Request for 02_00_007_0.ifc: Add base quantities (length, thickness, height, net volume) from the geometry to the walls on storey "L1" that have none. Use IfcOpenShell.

First a look at what the model holds.

```python
import ifcopenshell
import ifcopenshell.util.element
import ifcopenshell.util.unit

model = ifcopenshell.open("02_00_007_0.ifc")
print(model.schema)
for unit_type in ("LENGTHUNIT", "AREAUNIT", "VOLUMEUNIT"):
    print(unit_type, ifcopenshell.util.unit.calculate_unit_scale(model, unit_type))
storey = next(s for s in model.by_type("IfcBuildingStorey") if s.Name == "L1")
walls = [e for e in ifcopenshell.util.element.get_decomposition(storey) if e.is_a("IfcWall")]
for e in sorted(walls, key=lambda e: e.id()):
    print(e.id(), e.is_a(), e.Name, list(ifcopenshell.util.element.get_psets(e, qtos_only=True)), sep=" | ")
```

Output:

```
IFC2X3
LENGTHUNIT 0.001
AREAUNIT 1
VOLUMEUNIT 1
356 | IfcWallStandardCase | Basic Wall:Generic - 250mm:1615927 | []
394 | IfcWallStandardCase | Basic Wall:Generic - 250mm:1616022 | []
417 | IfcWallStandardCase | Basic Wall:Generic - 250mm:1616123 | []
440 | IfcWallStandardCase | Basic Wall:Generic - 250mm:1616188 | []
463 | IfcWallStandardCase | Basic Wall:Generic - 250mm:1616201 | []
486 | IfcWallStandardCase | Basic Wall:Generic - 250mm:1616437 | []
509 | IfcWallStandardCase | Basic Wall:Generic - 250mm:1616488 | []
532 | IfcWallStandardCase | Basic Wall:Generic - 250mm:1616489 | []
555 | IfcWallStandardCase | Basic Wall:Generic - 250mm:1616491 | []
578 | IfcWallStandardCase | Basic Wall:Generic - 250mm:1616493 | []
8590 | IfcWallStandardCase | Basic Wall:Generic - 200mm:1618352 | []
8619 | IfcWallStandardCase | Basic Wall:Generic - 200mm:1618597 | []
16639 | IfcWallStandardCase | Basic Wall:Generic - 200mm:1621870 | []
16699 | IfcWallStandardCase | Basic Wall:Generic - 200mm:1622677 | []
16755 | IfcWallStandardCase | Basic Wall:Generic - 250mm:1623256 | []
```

```python
import ifcopenshell
import ifcopenshell.api.pset
import ifcopenshell.geom
import ifcopenshell.util.element
import ifcopenshell.util.shape
import ifcopenshell.util.unit

model = ifcopenshell.open("02_00_007_0.ifc")
unit_scale = ifcopenshell.util.unit.calculate_unit_scale(model)
volume_scale = ifcopenshell.util.unit.calculate_unit_scale(model, "VOLUMEUNIT")
settings = ifcopenshell.geom.settings()

storey = next(s for s in model.by_type("IfcBuildingStorey") if s.Name == "L1")
walls = [e for e in ifcopenshell.util.element.get_decomposition(storey) if e.is_a("IfcWall")]

for e in sorted(walls, key=lambda e: e.id()):
    if ifcopenshell.util.element.get_psets(e, qtos_only=True, should_inherit=False):
        continue
    # Geometry comes back in metres, in the element's own axes.
    shape = ifcopenshell.geom.create_shape(settings, e)
    values = {
        "Length": ifcopenshell.util.shape.get_x(shape.geometry) / unit_scale,
        "Width": ifcopenshell.util.shape.get_y(shape.geometry) / unit_scale,
        "Height": ifcopenshell.util.shape.get_z(shape.geometry) / unit_scale,
        "NetVolume": ifcopenshell.util.shape.get_volume(shape.geometry) / volume_scale,
    }
    qto = ifcopenshell.api.pset.add_qto(model, product=e, name="BaseQuantities")
    ifcopenshell.api.pset.edit_qto(model, qto=qto, properties=values)
    print(e.id(), {k: round(v, 3) for k, v in values.items()})

model.write("02_00_007_0_updated.ifc")
```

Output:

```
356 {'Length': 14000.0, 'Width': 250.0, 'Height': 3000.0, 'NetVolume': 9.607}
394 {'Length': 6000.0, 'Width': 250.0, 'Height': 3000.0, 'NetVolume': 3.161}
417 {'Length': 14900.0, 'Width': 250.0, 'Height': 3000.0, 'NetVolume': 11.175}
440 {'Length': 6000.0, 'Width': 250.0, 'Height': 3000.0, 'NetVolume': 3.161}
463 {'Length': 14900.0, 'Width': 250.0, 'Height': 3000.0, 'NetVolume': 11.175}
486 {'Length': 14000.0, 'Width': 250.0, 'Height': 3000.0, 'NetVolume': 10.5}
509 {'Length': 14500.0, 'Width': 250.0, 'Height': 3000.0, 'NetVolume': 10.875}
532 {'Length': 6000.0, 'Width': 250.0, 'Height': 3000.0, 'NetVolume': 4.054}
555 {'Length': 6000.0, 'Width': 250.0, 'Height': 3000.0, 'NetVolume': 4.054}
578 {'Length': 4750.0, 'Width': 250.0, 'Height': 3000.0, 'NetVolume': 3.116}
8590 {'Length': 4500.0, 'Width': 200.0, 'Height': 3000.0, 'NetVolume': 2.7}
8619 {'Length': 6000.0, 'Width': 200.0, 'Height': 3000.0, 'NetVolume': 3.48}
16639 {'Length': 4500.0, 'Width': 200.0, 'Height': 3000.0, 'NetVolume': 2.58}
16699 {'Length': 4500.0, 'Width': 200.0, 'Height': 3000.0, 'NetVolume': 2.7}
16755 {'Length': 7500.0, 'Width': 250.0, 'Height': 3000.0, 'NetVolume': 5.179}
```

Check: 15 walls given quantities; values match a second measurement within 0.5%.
